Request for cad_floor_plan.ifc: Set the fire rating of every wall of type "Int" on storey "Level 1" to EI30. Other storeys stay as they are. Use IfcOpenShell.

First a look at what the model holds.

```python
import ifcopenshell
import ifcopenshell.util.element

model = ifcopenshell.open("cad_floor_plan.ifc")
print(model.schema)
storey = next(s for s in model.by_type("IfcBuildingStorey") if s.Name == "Level 1")
walls = [e for e in ifcopenshell.util.element.get_decomposition(storey) if e.is_a("IfcWall")]
seen = {}
for e in walls:
    element_type = ifcopenshell.util.element.get_type(e)
    key = (element_type.Name if element_type != e and element_type else None, ifcopenshell.util.element.get_pset(e, "Pset_WallCommon", "FireRating"))
    seen[key] = seen.get(key, 0) + 1
for (name, value), count in sorted(seen.items(), key=str):
    print(count, "x", name, "|", value)
```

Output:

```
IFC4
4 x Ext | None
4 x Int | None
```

```python
import ifcopenshell
import ifcopenshell.api.pset
import ifcopenshell.util.element

model = ifcopenshell.open("cad_floor_plan.ifc")

storey = next(s for s in model.by_type("IfcBuildingStorey") if s.Name == "Level 1")
walls = [e for e in ifcopenshell.util.element.get_decomposition(storey) if e.is_a("IfcWall")]

count = 0
for e in walls:
    element_type = ifcopenshell.util.element.get_type(e)
    if element_type in (None, e) or element_type.Name != "Int":
        continue
    # add_pset returns the element's existing set when there is one.
    pset = ifcopenshell.api.pset.add_pset(model, product=e, name="Pset_WallCommon")
    ifcopenshell.api.pset.edit_pset(model, pset=pset, properties={"FireRating": "EI30"})
    count += 1

print(count, "walls updated")

model.write("cad_floor_plan_v2.ifc")
```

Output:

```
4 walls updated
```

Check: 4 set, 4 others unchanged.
